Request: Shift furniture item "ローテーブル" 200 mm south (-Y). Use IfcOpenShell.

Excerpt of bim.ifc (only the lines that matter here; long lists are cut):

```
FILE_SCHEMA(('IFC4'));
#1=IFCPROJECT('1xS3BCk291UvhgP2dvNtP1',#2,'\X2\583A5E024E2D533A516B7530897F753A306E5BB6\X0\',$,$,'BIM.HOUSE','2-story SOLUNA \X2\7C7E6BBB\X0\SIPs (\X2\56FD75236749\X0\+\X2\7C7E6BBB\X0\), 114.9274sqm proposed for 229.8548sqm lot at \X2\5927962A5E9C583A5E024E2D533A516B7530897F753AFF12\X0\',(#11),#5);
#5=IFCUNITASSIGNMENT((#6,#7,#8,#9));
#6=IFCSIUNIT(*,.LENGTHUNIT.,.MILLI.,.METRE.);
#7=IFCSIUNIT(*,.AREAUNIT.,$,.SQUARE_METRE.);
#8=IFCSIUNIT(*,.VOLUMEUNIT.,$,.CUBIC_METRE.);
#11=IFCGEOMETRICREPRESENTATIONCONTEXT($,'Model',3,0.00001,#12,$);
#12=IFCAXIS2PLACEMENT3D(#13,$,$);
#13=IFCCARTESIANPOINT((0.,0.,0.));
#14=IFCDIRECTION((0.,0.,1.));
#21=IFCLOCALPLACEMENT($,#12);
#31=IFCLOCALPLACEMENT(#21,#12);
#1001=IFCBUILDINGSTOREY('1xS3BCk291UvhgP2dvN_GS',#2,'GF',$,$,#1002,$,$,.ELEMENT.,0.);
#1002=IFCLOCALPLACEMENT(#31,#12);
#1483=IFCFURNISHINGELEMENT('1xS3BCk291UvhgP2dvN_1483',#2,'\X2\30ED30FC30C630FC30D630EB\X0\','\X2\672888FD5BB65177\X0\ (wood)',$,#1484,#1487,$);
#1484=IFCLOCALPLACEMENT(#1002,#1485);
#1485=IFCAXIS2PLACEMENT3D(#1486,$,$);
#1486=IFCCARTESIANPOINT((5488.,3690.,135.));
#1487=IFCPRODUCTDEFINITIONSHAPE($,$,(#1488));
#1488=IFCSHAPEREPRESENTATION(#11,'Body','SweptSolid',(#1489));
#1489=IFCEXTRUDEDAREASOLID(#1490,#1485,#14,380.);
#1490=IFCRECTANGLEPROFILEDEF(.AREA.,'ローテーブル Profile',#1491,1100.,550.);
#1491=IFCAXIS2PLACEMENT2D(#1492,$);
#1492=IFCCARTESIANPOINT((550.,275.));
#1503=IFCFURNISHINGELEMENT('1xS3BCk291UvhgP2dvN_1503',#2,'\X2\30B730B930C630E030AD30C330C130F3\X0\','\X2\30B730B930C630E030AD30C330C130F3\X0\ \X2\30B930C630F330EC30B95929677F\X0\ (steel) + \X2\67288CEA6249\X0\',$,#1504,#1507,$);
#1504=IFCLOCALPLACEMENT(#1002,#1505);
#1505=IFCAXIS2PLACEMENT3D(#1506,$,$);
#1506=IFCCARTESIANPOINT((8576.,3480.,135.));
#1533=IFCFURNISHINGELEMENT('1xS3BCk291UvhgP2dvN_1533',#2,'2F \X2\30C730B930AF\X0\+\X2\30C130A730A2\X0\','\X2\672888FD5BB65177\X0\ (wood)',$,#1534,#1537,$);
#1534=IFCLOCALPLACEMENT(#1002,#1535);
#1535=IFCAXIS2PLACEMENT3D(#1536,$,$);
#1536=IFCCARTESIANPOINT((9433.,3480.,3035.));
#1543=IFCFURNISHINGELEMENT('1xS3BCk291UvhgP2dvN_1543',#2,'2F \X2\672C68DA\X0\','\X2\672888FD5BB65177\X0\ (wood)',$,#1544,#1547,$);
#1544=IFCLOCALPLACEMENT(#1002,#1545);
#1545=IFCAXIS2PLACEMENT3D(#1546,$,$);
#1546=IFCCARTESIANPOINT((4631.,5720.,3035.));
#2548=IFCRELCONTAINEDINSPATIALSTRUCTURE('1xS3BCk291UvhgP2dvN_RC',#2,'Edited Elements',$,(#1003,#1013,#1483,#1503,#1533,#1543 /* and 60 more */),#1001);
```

```python
import ifcopenshell
import ifcopenshell.api.geometry
import ifcopenshell.util.placement
import ifcopenshell.util.unit

model = ifcopenshell.open("bim.ifc")
unit_scale = ifcopenshell.util.unit.calculate_unit_scale(model)

item = model.by_id(1483)
matrix = ifcopenshell.util.placement.get_local_placement(item.ObjectPlacement)
matrix[1, 3] -= 0.2 / unit_scale
ifcopenshell.api.geometry.edit_object_placement(model, product=item, matrix=matrix, is_si=False)

print(ifcopenshell.util.placement.get_local_placement(item.ObjectPlacement).round(3) + 0.0)

model.write("bim_edited.ifc")
```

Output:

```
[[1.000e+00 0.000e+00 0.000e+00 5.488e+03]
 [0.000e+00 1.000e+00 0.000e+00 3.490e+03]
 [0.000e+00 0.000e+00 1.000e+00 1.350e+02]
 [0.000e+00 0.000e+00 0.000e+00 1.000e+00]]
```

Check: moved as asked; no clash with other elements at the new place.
